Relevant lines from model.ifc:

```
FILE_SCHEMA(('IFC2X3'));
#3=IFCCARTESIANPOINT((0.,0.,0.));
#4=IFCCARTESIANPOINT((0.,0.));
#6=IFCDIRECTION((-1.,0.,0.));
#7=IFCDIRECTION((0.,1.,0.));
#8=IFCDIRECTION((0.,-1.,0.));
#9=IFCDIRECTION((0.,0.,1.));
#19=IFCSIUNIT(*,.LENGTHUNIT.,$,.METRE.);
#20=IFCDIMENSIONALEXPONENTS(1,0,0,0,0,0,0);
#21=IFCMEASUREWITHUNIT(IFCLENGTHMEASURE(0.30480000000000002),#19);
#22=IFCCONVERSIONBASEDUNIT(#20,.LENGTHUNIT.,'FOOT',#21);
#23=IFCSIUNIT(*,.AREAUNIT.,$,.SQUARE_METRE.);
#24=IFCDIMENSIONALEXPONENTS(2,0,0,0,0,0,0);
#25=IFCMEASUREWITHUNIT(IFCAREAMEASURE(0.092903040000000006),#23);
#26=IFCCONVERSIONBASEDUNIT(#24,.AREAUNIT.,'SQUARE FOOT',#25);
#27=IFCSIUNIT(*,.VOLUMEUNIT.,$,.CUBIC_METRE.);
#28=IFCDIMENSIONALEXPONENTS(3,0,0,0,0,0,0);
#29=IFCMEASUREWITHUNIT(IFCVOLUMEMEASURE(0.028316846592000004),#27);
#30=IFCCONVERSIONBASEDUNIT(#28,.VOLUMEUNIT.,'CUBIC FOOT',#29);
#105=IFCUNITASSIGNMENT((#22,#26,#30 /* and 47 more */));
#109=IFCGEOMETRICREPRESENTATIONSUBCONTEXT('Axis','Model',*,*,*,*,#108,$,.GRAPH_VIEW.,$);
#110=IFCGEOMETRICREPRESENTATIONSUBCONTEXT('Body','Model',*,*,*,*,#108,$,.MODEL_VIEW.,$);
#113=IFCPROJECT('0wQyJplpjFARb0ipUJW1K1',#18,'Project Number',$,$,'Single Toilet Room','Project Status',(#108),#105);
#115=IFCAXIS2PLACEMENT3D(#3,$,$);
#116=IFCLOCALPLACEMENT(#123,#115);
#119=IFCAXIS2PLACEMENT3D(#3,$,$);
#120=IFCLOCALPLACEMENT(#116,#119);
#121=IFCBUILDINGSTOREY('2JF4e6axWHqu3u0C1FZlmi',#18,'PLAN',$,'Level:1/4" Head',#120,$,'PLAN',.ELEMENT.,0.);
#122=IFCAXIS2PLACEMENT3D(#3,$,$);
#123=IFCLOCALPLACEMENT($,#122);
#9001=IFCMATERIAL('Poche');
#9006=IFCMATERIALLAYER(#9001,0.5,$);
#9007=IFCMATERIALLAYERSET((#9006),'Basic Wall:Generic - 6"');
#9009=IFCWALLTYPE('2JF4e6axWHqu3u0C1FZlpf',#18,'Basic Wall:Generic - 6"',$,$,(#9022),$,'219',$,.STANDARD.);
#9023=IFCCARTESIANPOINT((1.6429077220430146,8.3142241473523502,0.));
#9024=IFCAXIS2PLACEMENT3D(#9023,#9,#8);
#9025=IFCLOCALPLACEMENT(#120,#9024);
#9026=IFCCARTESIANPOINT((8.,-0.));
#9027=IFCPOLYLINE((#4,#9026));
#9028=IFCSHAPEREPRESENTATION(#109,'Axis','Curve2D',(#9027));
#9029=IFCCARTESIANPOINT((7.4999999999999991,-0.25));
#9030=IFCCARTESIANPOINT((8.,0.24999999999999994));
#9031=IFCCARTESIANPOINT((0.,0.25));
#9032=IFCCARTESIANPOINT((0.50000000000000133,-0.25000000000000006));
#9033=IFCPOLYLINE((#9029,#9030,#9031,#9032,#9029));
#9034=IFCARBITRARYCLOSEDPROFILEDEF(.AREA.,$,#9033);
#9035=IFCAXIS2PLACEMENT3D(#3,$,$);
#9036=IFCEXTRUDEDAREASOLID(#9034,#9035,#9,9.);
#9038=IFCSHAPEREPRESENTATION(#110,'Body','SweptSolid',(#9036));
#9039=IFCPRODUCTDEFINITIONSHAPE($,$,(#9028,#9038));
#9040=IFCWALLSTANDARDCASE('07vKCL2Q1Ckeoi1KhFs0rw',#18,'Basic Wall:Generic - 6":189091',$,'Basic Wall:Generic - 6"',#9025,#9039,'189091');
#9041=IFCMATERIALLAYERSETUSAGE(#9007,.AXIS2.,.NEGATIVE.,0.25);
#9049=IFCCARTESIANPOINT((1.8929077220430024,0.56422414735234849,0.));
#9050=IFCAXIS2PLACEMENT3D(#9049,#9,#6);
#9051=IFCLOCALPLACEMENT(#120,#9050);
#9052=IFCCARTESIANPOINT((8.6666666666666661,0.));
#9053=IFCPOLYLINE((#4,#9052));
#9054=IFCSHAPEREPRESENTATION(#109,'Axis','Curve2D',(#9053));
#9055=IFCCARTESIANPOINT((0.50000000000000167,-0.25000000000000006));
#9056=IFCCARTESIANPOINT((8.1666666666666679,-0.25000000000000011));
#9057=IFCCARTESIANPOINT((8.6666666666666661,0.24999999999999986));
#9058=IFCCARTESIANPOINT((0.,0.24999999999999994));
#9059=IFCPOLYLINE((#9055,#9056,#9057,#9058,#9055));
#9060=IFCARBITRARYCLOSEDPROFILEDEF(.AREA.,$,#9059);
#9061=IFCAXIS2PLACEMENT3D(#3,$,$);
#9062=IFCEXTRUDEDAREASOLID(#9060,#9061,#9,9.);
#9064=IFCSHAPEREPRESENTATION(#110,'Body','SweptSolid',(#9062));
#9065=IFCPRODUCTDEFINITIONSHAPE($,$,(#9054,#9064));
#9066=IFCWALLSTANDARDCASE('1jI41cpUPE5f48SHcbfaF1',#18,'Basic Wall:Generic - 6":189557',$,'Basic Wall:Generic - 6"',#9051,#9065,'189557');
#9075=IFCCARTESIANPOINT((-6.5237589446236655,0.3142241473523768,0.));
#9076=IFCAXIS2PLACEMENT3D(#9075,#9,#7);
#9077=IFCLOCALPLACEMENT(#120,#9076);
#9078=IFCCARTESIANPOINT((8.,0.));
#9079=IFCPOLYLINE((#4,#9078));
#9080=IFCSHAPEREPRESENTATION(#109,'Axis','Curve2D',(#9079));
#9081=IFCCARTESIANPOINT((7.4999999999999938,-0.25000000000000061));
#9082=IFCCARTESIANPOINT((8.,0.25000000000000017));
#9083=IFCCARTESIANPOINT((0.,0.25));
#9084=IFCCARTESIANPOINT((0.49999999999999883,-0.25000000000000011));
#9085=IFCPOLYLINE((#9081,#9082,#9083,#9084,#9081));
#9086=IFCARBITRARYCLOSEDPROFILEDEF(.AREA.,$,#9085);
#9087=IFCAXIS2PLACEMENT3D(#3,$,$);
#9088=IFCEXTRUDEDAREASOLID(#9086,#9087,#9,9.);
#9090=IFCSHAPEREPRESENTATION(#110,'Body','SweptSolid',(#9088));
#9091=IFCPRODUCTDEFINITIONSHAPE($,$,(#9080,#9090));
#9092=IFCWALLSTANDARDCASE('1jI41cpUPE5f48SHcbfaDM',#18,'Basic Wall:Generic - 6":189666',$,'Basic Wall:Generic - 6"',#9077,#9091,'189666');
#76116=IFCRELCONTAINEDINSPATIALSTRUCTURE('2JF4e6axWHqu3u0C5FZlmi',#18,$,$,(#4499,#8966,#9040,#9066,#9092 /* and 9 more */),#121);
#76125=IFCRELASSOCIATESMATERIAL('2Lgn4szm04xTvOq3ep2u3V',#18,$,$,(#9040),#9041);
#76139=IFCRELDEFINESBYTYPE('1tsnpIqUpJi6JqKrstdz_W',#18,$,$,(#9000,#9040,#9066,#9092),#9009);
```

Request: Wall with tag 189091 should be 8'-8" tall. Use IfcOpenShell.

```python
import ifcopenshell
import ifcopenshell.geom
import ifcopenshell.util.representation
import ifcopenshell.util.shape
import ifcopenshell.util.unit

model = ifcopenshell.open("model.ifc")
unit_scale = ifcopenshell.util.unit.calculate_unit_scale(model)
settings = ifcopenshell.geom.settings()


def volume(element):
    """Net volume in cubic metres, openings subtracted."""
    shape = ifcopenshell.geom.create_shape(settings, element)
    return ifcopenshell.util.shape.get_volume(shape.geometry)


wall = model.by_guid("07vKCL2Q1Ckeoi1KhFs0rw")
before = volume(wall)

body = ifcopenshell.util.representation.get_representation(wall, "Model", "Body")
solid = body.Items[0]
old_height = solid.Depth
solid.Depth = 104 * 0.0254 / unit_scale
after = volume(wall)

print(f"height {old_height:g} -> {solid.Depth:g}, volume {before:.3f} -> {after:.3f} m3")

model.write("model_rev.ifc")
```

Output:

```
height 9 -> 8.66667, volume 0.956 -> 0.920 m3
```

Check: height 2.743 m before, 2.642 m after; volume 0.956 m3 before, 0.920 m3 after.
